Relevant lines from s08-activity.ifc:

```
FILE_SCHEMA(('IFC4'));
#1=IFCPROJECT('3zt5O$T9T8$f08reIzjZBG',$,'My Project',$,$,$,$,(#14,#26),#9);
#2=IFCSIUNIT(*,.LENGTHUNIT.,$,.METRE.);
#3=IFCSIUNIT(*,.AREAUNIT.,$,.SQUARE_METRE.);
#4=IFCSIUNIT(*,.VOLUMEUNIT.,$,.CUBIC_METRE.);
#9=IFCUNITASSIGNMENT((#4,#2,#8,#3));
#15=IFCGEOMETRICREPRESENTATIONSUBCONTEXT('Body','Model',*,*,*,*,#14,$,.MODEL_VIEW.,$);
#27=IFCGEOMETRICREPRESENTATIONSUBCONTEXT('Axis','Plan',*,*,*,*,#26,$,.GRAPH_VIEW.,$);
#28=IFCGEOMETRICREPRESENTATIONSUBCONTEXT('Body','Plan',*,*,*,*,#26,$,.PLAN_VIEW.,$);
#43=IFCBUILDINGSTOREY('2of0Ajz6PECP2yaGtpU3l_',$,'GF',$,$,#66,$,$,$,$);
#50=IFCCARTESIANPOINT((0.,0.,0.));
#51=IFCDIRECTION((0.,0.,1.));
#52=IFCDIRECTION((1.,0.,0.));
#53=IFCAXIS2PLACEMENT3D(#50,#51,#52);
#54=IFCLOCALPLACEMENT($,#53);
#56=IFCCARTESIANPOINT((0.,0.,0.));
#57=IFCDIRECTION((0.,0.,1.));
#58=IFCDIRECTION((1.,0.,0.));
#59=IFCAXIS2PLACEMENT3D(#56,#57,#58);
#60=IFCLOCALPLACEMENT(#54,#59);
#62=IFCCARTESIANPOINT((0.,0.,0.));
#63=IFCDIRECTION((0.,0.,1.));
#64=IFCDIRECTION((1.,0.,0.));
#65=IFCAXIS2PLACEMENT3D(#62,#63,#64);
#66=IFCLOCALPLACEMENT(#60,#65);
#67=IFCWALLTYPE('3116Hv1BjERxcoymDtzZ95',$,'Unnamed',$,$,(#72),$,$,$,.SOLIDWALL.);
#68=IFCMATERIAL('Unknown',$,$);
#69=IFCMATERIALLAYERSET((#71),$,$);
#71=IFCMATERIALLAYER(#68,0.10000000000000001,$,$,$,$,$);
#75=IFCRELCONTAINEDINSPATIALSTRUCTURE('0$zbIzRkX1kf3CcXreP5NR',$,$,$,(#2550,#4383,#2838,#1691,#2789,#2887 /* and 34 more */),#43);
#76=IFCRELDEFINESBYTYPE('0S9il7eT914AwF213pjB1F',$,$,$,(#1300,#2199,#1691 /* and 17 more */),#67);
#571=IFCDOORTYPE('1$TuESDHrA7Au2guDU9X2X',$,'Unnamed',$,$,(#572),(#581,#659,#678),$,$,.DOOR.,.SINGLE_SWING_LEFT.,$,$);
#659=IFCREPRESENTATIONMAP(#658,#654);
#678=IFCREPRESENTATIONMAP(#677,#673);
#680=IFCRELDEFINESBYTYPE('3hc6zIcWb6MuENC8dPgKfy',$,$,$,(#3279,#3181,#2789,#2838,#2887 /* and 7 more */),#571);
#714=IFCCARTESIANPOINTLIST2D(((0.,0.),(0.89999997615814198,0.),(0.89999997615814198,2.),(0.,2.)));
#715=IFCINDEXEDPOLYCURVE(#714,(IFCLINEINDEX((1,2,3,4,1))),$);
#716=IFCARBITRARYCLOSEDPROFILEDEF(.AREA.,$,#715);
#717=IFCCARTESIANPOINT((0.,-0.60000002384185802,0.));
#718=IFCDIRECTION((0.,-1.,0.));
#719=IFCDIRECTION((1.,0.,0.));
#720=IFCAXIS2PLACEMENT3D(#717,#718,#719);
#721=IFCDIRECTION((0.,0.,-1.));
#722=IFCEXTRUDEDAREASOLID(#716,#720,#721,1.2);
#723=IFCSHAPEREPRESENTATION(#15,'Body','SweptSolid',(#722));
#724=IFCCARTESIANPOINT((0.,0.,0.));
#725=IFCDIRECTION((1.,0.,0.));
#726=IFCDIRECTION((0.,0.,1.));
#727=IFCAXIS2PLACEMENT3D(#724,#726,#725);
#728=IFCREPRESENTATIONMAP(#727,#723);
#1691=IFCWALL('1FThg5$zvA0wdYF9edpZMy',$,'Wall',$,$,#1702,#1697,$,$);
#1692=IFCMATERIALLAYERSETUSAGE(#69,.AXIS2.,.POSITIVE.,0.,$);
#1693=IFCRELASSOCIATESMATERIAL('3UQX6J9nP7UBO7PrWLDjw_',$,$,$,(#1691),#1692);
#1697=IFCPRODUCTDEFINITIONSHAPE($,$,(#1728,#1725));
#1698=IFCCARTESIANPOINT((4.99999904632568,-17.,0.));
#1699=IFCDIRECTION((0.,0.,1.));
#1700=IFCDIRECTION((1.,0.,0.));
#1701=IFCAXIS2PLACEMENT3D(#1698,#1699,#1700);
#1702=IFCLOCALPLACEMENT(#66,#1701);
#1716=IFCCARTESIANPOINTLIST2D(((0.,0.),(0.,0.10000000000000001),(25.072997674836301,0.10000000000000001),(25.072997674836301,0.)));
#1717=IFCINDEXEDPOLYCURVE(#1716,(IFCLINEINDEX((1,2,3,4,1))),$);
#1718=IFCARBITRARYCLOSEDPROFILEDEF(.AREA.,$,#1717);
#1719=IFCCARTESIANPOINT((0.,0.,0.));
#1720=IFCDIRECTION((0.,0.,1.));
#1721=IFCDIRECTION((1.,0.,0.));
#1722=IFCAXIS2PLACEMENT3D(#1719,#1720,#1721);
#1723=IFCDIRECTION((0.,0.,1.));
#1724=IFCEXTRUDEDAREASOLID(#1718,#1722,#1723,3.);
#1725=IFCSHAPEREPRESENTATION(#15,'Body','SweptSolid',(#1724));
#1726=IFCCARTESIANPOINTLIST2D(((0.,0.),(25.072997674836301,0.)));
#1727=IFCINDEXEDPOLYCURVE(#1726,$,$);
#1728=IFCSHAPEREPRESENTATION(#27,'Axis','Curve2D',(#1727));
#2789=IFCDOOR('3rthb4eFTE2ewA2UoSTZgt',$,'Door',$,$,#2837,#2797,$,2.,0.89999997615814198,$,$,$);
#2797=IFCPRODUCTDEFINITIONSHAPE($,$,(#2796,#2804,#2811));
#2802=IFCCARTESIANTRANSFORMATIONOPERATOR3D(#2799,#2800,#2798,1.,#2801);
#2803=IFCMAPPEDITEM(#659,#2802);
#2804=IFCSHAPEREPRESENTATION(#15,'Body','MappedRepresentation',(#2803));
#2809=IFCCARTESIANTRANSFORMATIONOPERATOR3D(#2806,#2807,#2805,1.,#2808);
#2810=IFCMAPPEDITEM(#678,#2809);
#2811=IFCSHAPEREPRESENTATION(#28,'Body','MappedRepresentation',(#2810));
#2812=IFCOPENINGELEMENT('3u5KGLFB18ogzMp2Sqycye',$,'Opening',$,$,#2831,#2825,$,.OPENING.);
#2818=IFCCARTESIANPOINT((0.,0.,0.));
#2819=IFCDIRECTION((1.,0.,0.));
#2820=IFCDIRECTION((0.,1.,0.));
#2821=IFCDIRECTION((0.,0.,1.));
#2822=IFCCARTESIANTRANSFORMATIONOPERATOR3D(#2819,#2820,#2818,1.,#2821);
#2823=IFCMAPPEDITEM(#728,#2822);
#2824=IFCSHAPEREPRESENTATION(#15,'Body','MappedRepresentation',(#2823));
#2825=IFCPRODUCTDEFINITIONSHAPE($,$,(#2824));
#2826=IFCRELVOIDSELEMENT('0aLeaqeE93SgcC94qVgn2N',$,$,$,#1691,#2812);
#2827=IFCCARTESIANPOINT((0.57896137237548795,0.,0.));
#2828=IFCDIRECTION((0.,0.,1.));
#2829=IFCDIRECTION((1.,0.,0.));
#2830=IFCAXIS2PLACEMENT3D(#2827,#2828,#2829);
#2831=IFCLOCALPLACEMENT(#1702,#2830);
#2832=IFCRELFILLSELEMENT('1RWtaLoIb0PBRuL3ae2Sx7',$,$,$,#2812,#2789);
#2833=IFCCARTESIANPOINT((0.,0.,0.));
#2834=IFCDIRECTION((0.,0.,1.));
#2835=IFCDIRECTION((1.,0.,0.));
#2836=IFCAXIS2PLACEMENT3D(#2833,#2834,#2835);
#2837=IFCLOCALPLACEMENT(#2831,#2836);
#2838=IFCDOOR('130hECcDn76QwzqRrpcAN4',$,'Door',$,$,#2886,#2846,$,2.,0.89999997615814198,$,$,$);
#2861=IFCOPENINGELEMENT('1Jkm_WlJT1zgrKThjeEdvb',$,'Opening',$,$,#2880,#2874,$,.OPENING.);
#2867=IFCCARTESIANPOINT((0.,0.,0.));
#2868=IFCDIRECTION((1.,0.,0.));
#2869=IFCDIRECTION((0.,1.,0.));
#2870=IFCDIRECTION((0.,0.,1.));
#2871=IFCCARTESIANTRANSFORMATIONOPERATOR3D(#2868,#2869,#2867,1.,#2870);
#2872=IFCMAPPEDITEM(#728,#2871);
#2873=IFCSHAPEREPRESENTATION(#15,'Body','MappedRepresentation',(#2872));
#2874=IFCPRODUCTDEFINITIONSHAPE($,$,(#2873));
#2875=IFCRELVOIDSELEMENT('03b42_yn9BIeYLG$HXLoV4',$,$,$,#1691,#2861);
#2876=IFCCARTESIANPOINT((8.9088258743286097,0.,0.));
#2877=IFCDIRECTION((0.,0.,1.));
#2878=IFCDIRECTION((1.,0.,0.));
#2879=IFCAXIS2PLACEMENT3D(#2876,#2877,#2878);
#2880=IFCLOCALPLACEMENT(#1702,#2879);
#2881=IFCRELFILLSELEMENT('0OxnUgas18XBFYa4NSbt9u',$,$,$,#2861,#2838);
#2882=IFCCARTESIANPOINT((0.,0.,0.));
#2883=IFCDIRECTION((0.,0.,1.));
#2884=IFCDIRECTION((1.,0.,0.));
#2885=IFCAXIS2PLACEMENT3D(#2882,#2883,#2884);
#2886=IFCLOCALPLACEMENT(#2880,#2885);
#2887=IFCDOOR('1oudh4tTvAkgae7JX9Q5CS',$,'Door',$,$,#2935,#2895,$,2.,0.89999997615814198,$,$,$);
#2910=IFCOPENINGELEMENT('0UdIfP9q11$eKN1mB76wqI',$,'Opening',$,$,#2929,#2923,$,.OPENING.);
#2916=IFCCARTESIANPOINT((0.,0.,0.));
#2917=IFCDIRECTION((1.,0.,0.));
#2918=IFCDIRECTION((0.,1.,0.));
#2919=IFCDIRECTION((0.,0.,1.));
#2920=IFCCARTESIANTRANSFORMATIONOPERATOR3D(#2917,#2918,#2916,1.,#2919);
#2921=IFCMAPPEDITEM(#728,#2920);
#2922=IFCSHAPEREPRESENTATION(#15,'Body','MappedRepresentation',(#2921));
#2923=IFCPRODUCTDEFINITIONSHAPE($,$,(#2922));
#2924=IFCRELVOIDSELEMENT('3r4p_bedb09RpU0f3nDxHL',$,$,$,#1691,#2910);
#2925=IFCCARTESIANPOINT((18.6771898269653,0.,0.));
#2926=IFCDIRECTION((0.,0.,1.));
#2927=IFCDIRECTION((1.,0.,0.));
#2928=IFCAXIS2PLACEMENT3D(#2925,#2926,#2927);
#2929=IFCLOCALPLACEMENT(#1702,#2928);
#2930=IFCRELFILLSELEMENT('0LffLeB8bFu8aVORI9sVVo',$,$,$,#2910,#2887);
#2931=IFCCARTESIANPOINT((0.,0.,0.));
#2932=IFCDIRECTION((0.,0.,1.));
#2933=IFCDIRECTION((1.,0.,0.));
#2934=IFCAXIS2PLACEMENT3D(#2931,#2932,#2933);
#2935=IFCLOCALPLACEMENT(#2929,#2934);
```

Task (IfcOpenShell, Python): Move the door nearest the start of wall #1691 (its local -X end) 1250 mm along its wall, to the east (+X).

```python
import ifcopenshell
import ifcopenshell.api.geometry
import ifcopenshell.util.placement
import ifcopenshell.util.unit

model = ifcopenshell.open("s08-activity.ifc")
unit_scale = ifcopenshell.util.unit.calculate_unit_scale(model)

door = model.by_guid("3rthb4eFTE2ewA2UoSTZgt")
opening = door.FillsVoids[0].RelatingOpeningElement
wall = opening.VoidsElements[0].RelatingBuildingElement

wall_matrix = ifcopenshell.util.placement.get_local_placement(wall.ObjectPlacement)
shift = wall_matrix[:3, 0] * 1.25 / unit_scale
before = ifcopenshell.util.placement.get_local_placement(door.ObjectPlacement)[:3, 3].copy()

# The door is placed relative to its opening, so it follows when the opening moves.
matrix = ifcopenshell.util.placement.get_local_placement(opening.ObjectPlacement)
matrix[:3, 3] += shift
ifcopenshell.api.geometry.edit_object_placement(
    model, product=opening, matrix=matrix, is_si=False, should_transform_children=True
)

after = ifcopenshell.util.placement.get_local_placement(door.ObjectPlacement)[:3, 3]
print("door moved by", (after - before).round(3) + 0.0)

model.write("s08-activity-out.ifc")
```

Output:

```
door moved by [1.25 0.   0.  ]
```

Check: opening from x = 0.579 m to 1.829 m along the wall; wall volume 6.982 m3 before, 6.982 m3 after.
